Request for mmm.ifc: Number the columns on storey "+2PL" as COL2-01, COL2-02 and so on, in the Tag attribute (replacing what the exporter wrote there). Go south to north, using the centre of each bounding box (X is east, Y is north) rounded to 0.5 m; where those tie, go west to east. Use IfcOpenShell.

First a look at what the model holds.

```python
import ifcopenshell
import ifcopenshell.util.element
import ifcopenshell.util.placement

model = ifcopenshell.open("mmm.ifc")
print(model.schema)
storey = next(s for s in model.by_type("IfcBuildingStorey") if s.Name == "+2PL")
columns = [e for e in ifcopenshell.util.element.get_decomposition(storey) if e.is_a("IfcColumn")]
for e in sorted(columns, key=lambda e: e.id()):
    origin = ifcopenshell.util.placement.get_local_placement(e.ObjectPlacement)[:3, 3]
    print(e.id(), e.Tag, e.Name, origin.round(2) + 0.0, sep=" | ")
```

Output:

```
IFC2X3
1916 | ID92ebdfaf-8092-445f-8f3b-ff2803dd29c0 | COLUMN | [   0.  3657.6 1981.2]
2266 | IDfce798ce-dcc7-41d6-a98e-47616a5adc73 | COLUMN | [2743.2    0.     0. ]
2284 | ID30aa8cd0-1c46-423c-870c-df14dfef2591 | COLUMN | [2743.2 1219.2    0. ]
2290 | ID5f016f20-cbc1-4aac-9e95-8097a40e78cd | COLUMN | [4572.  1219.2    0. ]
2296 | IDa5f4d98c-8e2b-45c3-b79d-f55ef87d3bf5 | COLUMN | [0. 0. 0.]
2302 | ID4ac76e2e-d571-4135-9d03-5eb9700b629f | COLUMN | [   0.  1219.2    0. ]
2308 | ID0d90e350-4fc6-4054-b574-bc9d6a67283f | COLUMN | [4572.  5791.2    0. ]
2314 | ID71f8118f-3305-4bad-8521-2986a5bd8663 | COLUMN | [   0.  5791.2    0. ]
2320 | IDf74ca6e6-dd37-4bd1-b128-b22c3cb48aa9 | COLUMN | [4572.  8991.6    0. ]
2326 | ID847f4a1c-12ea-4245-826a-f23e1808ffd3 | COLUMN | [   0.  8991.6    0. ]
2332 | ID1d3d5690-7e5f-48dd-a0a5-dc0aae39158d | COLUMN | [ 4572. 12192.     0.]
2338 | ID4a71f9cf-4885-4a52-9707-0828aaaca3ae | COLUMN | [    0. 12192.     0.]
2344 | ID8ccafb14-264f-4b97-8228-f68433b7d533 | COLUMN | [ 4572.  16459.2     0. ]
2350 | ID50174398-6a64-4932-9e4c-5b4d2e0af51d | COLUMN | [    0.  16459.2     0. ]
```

```python
import ifcopenshell
import ifcopenshell.geom
import ifcopenshell.util.element
import ifcopenshell.util.shape

model = ifcopenshell.open("mmm.ifc")
settings = ifcopenshell.geom.settings()
settings.set("use-world-coords", True)


def centre(element):
    shape = ifcopenshell.geom.create_shape(settings, element)
    return ifcopenshell.util.shape.get_bbox_centroid(shape.geometry)


storey = next(s for s in model.by_type("IfcBuildingStorey") if s.Name == "+2PL")
columns = [e for e in ifcopenshell.util.element.get_decomposition(storey) if e.is_a("IfcColumn")]

# Insertion points can sit at a corner or the storey origin, so sort by the geometry (in metres).
centres = {e: centre(e) for e in columns}
columns.sort(key=lambda e: (round(centres[e][1] / 0.5), centres[e][0]))

for i, e in enumerate(columns, start=1):
    number = f"COL2-{i:02d}"
    e.Tag = number
    print(e.id(), number)

model.write("mmm_v2.ifc")
```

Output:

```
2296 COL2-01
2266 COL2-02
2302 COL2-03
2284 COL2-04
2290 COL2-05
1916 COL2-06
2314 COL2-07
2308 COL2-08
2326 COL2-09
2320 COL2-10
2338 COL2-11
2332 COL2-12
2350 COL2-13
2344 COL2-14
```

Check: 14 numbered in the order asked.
